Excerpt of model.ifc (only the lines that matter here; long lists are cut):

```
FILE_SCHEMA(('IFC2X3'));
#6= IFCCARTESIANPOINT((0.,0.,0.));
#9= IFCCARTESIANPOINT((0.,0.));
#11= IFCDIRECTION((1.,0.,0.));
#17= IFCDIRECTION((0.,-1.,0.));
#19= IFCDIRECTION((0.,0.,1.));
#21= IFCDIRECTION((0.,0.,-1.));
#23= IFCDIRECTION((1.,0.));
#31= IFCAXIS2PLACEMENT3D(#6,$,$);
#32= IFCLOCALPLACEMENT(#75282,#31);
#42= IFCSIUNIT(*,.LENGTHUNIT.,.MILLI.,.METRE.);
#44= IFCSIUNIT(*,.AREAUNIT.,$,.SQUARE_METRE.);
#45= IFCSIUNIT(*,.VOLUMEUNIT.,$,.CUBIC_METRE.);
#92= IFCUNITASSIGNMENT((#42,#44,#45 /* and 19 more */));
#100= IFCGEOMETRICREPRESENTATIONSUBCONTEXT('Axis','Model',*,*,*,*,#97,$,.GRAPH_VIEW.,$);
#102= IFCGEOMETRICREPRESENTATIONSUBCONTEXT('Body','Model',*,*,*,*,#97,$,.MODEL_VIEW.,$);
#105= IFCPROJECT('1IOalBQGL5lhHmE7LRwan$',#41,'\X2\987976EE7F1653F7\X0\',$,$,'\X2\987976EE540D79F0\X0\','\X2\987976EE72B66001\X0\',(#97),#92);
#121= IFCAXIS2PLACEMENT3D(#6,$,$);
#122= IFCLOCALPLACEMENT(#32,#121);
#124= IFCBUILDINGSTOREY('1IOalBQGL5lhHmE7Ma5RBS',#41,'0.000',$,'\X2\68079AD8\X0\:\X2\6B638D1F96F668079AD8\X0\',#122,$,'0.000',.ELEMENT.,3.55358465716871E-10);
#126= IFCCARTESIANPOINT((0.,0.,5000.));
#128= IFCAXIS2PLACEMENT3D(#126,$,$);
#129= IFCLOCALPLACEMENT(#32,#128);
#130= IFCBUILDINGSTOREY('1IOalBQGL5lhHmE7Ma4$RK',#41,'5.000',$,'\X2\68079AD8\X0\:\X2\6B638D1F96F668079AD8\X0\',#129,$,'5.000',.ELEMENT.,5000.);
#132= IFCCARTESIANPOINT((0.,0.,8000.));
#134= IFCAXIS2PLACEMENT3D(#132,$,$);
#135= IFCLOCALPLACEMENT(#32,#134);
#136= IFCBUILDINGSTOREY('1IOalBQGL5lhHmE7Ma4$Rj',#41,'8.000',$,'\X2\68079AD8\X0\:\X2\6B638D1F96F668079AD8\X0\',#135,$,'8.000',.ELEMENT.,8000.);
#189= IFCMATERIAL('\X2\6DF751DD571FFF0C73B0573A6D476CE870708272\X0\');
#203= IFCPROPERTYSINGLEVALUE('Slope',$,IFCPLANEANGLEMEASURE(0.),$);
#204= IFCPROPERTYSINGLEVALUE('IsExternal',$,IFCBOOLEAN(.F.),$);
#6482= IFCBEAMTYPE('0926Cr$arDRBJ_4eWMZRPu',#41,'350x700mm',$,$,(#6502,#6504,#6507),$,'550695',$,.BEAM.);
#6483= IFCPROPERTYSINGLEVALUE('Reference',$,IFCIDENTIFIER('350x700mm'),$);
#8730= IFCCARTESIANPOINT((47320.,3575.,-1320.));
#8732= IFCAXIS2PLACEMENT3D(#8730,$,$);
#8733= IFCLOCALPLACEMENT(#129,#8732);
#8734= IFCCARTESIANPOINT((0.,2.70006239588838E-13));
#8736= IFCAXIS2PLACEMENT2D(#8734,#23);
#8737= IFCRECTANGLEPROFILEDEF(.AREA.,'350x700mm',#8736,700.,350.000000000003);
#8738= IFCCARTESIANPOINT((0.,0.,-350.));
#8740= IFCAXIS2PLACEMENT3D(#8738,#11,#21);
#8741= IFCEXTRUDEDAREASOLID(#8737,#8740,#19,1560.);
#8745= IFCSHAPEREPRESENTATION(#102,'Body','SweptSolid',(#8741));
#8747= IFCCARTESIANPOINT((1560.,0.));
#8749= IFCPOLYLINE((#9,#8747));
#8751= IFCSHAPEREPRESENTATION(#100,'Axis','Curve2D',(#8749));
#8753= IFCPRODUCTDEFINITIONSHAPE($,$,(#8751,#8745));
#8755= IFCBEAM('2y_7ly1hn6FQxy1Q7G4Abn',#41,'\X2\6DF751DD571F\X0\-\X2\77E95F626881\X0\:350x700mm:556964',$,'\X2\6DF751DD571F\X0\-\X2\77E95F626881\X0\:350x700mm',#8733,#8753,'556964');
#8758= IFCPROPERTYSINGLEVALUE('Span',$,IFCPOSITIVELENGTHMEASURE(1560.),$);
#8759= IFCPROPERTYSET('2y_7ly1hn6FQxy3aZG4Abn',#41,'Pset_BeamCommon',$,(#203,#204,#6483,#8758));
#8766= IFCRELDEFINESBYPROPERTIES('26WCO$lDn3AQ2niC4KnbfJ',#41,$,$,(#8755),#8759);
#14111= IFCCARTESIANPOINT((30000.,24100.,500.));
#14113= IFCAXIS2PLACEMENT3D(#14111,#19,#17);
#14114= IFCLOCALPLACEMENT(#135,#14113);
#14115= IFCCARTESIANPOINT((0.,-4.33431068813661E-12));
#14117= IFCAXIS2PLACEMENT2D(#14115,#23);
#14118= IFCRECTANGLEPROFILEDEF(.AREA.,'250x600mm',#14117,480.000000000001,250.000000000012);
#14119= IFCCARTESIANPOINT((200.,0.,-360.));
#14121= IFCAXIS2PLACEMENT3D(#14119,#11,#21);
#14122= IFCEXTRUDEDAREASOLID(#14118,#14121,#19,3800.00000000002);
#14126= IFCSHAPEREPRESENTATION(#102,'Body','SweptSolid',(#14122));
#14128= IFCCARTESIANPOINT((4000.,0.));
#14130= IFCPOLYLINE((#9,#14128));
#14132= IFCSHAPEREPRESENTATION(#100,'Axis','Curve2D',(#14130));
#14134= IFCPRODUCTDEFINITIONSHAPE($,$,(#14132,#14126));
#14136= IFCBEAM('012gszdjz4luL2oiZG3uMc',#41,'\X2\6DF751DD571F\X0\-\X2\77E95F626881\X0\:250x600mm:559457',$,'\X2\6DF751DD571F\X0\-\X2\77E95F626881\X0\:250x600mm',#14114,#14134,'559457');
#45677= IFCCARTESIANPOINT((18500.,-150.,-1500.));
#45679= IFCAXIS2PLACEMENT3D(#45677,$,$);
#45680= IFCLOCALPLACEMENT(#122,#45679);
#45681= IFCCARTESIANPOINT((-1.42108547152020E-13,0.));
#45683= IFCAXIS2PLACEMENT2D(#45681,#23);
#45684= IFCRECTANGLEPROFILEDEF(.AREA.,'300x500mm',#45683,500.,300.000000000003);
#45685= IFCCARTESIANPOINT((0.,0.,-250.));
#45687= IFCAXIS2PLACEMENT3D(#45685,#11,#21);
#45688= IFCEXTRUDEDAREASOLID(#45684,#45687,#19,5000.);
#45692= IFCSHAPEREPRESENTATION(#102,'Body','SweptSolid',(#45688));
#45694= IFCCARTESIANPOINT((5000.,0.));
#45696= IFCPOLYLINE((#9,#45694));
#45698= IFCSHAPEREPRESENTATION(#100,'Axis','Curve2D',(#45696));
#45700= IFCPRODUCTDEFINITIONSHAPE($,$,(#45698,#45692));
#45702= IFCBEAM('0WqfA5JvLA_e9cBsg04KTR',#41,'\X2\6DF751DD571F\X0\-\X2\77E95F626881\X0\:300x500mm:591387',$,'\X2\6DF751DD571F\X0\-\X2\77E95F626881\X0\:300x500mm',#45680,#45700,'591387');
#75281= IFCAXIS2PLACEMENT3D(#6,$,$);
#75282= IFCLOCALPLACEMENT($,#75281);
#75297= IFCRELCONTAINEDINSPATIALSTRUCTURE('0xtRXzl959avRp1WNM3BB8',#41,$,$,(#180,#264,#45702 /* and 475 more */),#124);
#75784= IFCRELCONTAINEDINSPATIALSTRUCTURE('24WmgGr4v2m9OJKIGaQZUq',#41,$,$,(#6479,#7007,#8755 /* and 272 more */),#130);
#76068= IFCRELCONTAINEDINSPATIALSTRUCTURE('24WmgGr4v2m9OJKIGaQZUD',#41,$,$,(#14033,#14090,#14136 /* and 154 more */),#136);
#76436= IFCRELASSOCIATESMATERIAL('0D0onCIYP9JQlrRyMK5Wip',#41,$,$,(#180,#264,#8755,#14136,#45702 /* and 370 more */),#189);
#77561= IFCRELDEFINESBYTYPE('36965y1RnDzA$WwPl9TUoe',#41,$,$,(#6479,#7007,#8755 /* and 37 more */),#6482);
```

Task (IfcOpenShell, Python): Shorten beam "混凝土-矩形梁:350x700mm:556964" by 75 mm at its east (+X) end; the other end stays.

```python
import numpy as np
import ifcopenshell
import ifcopenshell.api.pset
import ifcopenshell.util.element
import ifcopenshell.util.representation
import ifcopenshell.util.unit

model = ifcopenshell.open("model.ifc")
unit_scale = ifcopenshell.util.unit.calculate_unit_scale(model)

member = model.by_guid("2y_7ly1hn6FQxy1Q7G4Abn")
change = -0.075 / unit_scale

# The extrusion runs towards the end named, so only its depth changes.
body = ifcopenshell.util.representation.get_representation(member, "Model", "Body")
solid = body.Items[0]
old_length = solid.Depth
solid.Depth += change

# Move the axis end point with it.
axis = next(r for r in member.Representation.Representations if r.RepresentationIdentifier == "Axis").Items[0]
start, end = (np.array(p.Coordinates) for p in axis.Points)
end = end + (end - start) / np.linalg.norm(end - start) * change
point = model.createIfcCartesianPoint(end.tolist())
axis.Points = [axis.Points[0], point]

# Update the stored length and volume.
pset = model.by_id(ifcopenshell.util.element.get_pset(member, "Pset_BeamCommon", should_inherit=False)["id"])
ifcopenshell.api.pset.edit_pset(model, pset=pset, properties={
    "Span": model.create_entity("IfcPositiveLengthMeasure", solid.Depth),
})

print(f"length {old_length:g} -> {solid.Depth:g}")

model.write("model_updated.ifc")
```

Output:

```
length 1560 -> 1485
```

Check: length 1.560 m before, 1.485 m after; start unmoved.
